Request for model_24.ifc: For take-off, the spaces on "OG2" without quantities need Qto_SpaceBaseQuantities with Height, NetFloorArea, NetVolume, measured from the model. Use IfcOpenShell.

First a look at what the model holds.

```python
import ifcopenshell
import ifcopenshell.util.element
import ifcopenshell.util.unit

model = ifcopenshell.open("model_24.ifc")
print(model.schema)
for unit_type in ("LENGTHUNIT", "AREAUNIT", "VOLUMEUNIT"):
    print(unit_type, ifcopenshell.util.unit.calculate_unit_scale(model, unit_type))
storey = next(s for s in model.by_type("IfcBuildingStorey") if s.Name == "OG2")
spaces = [e for e in ifcopenshell.util.element.get_decomposition(storey) if e.is_a("IfcSpace")]
for e in sorted(spaces, key=lambda e: e.id()):
    print(e.id(), e.is_a(), e.Name, list(ifcopenshell.util.element.get_psets(e, qtos_only=True)), sep=" | ")
```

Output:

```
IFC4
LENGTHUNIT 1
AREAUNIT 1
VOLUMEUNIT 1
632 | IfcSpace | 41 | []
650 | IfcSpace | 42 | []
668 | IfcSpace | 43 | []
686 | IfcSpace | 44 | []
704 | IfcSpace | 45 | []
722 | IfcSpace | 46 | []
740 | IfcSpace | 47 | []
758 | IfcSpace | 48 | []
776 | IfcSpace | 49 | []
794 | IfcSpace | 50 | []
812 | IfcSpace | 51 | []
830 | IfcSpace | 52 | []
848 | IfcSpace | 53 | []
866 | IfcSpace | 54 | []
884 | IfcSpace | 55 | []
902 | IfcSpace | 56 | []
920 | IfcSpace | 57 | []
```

```python
import ifcopenshell
import ifcopenshell.api.pset
import ifcopenshell.geom
import ifcopenshell.util.element
import ifcopenshell.util.shape
import ifcopenshell.util.unit

model = ifcopenshell.open("model_24.ifc")
unit_scale = ifcopenshell.util.unit.calculate_unit_scale(model)
area_scale = ifcopenshell.util.unit.calculate_unit_scale(model, "AREAUNIT")
volume_scale = ifcopenshell.util.unit.calculate_unit_scale(model, "VOLUMEUNIT")
settings = ifcopenshell.geom.settings()

storey = next(s for s in model.by_type("IfcBuildingStorey") if s.Name == "OG2")
spaces = [e for e in ifcopenshell.util.element.get_decomposition(storey) if e.is_a("IfcSpace")]

for e in sorted(spaces, key=lambda e: e.id()):
    if ifcopenshell.util.element.get_psets(e, qtos_only=True, should_inherit=False):
        continue
    # Geometry comes back in metres, in the element's own axes.
    shape = ifcopenshell.geom.create_shape(settings, e)
    values = {
        "Height": ifcopenshell.util.shape.get_z(shape.geometry) / unit_scale,
        "NetFloorArea": ifcopenshell.util.shape.get_footprint_area(shape.geometry) / area_scale,
        "NetVolume": ifcopenshell.util.shape.get_volume(shape.geometry) / volume_scale,
    }
    qto = ifcopenshell.api.pset.add_qto(model, product=e, name="Qto_SpaceBaseQuantities")
    ifcopenshell.api.pset.edit_qto(model, qto=qto, properties=values)
    print(e.id(), {k: round(v, 3) for k, v in values.items()})

model.write("model_24-out.ifc")
```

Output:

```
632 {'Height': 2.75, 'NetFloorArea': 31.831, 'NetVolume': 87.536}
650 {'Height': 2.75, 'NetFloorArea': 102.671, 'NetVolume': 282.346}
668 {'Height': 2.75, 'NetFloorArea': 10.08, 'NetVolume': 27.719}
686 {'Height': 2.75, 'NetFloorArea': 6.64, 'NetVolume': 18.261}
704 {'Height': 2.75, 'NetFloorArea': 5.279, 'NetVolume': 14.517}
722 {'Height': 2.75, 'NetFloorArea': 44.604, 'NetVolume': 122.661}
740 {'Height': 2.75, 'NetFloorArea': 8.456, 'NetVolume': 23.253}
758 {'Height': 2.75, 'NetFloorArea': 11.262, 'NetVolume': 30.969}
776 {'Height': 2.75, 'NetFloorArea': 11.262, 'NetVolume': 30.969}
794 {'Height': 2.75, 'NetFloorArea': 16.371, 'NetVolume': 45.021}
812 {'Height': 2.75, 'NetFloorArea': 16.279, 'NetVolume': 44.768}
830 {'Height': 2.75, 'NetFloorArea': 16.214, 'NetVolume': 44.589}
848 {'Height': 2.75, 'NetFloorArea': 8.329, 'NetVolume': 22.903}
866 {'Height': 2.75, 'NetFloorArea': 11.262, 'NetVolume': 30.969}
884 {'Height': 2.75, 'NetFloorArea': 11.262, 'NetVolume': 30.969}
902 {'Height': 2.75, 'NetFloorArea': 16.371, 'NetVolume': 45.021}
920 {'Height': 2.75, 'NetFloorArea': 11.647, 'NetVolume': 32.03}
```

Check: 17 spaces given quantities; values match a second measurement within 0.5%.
